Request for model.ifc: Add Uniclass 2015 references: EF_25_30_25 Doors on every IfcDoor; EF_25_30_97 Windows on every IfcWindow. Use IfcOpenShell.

First a look at what the model holds.

```python
import ifcopenshell

model = ifcopenshell.open("model.ifc")
print(model.schema)
print("classifications:", [c.Name for c in model.by_type("IfcClassification")])
for ifc_class in ("IfcDoor", "IfcRoof", "IfcStair", "IfcWall", "IfcWindow"):
    print(ifc_class, len(model.by_type(ifc_class)))
```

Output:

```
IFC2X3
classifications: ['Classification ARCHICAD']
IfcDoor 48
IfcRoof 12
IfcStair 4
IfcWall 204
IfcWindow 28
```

```python
import ifcopenshell
import ifcopenshell.api.classification

model = ifcopenshell.open("model.ifc")

# IFC2X3 requires Source and Edition and has no link from the project to the system.
system = model.create_entity("IfcClassification", Source="NBS", Edition="2015", Name="Uniclass 2015")

codes = {
    "IfcDoor": ("EF_25_30_25", "Doors"),
    "IfcWindow": ("EF_25_30_97", "Windows"),
}
for ifc_class, (code, name) in codes.items():
    products = model.by_type(ifc_class)
    ifcopenshell.api.classification.add_reference(
        model, products=products, classification=system, identification=code, name=name
    )
    print(code, len(products))

model.write("model_v2.ifc")
```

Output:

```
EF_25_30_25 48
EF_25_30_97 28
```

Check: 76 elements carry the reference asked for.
